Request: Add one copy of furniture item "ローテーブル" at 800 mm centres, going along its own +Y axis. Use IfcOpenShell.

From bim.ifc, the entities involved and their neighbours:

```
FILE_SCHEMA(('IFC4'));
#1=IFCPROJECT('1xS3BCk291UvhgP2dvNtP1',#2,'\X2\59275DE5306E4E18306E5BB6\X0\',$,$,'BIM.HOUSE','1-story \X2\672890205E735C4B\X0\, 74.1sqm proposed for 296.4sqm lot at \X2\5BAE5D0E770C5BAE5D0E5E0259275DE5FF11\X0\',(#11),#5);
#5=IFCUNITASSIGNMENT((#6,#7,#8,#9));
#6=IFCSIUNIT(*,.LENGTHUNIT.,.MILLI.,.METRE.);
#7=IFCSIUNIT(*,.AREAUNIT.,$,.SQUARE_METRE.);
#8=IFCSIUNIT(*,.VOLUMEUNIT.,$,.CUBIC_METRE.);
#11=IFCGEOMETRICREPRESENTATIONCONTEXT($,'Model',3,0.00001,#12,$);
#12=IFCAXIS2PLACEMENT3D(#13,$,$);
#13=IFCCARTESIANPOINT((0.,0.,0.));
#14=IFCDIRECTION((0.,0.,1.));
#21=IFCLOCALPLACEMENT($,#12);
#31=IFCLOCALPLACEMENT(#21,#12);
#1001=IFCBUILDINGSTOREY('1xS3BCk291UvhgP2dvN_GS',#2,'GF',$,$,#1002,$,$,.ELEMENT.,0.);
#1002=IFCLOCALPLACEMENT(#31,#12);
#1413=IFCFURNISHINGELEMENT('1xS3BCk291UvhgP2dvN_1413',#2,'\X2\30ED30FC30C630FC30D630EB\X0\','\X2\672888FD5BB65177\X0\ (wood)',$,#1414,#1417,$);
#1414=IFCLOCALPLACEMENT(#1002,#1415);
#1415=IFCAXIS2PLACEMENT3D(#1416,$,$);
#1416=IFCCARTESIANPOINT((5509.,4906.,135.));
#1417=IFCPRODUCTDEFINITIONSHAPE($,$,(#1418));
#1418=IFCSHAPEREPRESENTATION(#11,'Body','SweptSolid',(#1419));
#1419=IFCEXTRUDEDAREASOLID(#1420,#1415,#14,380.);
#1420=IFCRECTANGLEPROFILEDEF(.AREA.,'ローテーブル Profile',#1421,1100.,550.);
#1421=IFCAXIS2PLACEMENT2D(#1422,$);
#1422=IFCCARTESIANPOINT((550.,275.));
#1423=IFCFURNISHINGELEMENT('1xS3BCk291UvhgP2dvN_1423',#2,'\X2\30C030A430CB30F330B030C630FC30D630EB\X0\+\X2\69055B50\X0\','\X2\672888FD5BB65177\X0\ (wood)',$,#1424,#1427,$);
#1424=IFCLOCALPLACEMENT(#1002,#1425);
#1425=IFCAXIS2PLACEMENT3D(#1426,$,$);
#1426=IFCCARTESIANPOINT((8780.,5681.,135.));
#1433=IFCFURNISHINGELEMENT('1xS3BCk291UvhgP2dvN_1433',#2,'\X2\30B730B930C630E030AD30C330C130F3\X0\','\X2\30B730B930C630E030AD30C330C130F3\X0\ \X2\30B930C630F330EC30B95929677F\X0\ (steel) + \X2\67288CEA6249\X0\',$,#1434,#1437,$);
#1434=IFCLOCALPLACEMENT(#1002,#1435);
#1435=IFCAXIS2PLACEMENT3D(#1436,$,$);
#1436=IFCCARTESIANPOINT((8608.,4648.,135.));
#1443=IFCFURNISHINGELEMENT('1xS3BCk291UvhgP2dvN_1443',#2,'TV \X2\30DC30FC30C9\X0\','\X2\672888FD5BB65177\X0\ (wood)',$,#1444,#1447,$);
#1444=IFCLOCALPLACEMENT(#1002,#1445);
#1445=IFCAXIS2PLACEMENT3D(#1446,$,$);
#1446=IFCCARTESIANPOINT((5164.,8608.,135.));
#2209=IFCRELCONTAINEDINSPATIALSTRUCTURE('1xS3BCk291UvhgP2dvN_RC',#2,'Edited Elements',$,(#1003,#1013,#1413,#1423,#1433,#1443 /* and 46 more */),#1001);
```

```python
import ifcopenshell
import ifcopenshell.api.geometry
import ifcopenshell.api.root
import ifcopenshell.util.element
import ifcopenshell.util.placement
import ifcopenshell.util.unit

model = ifcopenshell.open("bim.ifc")
unit_scale = ifcopenshell.util.unit.calculate_unit_scale(model)


def reuse_history(source, copy):
    """copy_class also copies each property set's owner history, people and application; keep the originals."""
    for rel in copy.IsDefinedBy:
        if rel.is_a("IfcRelDefinesByProperties") and (history := rel.RelatingPropertyDefinition.OwnerHistory):
            rel.RelatingPropertyDefinition.OwnerHistory = source.OwnerHistory
            ifcopenshell.util.element.remove_deep2(model, history)


source = model.by_guid("1xS3BCk291UvhgP2dvN_1413")
base = ifcopenshell.util.placement.get_local_placement(source.ObjectPlacement)
step = base[:3, 1] * 0.8 / unit_scale

for i in range(1, 2):
    copy = ifcopenshell.api.root.copy_class(model, product=source)
    copy.Representation = ifcopenshell.util.element.copy_deep(
        model, source.Representation, exclude=["IfcGeometricRepresentationContext", "IfcRepresentationMap"]
    )
    reuse_history(source, copy)
    matrix = base.copy()
    matrix[:3, 3] += i * step
    print("added at", matrix[:3, 3].round(3) + 0.0)
    ifcopenshell.api.geometry.edit_object_placement(model, product=copy, matrix=matrix, is_si=False)

model.write("bim_v2.ifc")
```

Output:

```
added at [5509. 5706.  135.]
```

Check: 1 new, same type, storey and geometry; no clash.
